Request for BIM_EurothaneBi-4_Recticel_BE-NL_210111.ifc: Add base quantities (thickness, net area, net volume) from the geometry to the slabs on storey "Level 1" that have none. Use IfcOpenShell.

First a look at what the model holds.

```python
import ifcopenshell
import ifcopenshell.util.element
import ifcopenshell.util.unit

model = ifcopenshell.open("BIM_EurothaneBi-4_Recticel_BE-NL_210111.ifc")
print(model.schema)
for unit_type in ("LENGTHUNIT", "AREAUNIT", "VOLUMEUNIT"):
    print(unit_type, ifcopenshell.util.unit.calculate_unit_scale(model, unit_type))
storey = next(s for s in model.by_type("IfcBuildingStorey") if s.Name == "Level 1")
slabs = [e for e in ifcopenshell.util.element.get_decomposition(storey) if e.is_a("IfcSlab")]
for e in sorted(slabs, key=lambda e: e.id()):
    print(e.id(), e.is_a(), e.Name, list(ifcopenshell.util.element.get_psets(e, qtos_only=True)), sep=" | ")
```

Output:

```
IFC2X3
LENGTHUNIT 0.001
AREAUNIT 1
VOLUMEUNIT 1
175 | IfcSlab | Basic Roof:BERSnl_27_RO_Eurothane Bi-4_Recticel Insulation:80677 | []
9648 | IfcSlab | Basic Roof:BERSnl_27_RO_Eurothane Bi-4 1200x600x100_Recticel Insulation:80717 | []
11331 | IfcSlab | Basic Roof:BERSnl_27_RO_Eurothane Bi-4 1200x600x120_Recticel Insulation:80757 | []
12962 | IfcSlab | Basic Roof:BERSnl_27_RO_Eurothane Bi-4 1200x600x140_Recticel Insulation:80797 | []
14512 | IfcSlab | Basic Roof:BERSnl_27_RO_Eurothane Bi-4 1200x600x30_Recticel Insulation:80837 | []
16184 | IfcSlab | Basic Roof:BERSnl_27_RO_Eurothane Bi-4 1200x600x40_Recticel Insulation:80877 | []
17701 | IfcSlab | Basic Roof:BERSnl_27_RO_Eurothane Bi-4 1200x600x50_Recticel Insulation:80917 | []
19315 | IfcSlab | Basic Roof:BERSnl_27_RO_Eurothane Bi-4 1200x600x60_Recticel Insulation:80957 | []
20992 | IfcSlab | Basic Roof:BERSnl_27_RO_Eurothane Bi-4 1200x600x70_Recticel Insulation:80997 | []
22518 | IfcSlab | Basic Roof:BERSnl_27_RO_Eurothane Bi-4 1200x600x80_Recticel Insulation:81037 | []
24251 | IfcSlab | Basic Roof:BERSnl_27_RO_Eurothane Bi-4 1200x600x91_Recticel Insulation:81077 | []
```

```python
import ifcopenshell
import ifcopenshell.api.pset
import ifcopenshell.geom
import ifcopenshell.util.element
import ifcopenshell.util.shape
import ifcopenshell.util.unit

model = ifcopenshell.open("BIM_EurothaneBi-4_Recticel_BE-NL_210111.ifc")
unit_scale = ifcopenshell.util.unit.calculate_unit_scale(model)
area_scale = ifcopenshell.util.unit.calculate_unit_scale(model, "AREAUNIT")
volume_scale = ifcopenshell.util.unit.calculate_unit_scale(model, "VOLUMEUNIT")
settings = ifcopenshell.geom.settings()

storey = next(s for s in model.by_type("IfcBuildingStorey") if s.Name == "Level 1")
slabs = [e for e in ifcopenshell.util.element.get_decomposition(storey) if e.is_a("IfcSlab")]

for e in sorted(slabs, key=lambda e: e.id()):
    if ifcopenshell.util.element.get_psets(e, qtos_only=True, should_inherit=False):
        continue
    # Geometry comes back in metres, in the element's own axes.
    shape = ifcopenshell.geom.create_shape(settings, e)
    values = {
        "Width": ifcopenshell.util.shape.get_z(shape.geometry) / unit_scale,
        "NetArea": ifcopenshell.util.shape.get_footprint_area(shape.geometry) / area_scale,
        "NetVolume": ifcopenshell.util.shape.get_volume(shape.geometry) / volume_scale,
    }
    qto = ifcopenshell.api.pset.add_qto(model, product=e, name="BaseQuantities")
    ifcopenshell.api.pset.edit_qto(model, qto=qto, properties=values)
    print(e.id(), {k: round(v, 3) for k, v in values.items()})

model.write("BIM_EurothaneBi-4_Recticel_BE-NL_210111_updated.ifc")
```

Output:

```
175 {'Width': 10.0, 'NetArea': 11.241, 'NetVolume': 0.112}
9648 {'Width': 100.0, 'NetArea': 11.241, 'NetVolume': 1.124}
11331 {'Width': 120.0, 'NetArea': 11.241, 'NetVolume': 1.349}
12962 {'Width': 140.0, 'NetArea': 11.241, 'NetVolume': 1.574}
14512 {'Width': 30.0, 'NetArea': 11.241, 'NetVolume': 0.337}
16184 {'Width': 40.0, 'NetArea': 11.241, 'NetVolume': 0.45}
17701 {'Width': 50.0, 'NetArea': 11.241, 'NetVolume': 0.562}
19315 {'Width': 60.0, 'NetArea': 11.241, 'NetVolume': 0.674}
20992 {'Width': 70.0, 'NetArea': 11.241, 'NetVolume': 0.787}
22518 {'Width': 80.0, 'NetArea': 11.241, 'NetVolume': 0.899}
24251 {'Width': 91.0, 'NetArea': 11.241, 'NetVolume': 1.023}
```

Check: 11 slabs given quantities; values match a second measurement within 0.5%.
